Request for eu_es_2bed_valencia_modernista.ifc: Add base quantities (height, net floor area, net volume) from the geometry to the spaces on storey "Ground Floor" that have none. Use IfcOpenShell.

First a look at what the model holds.

```python
import ifcopenshell
import ifcopenshell.util.element
import ifcopenshell.util.unit

model = ifcopenshell.open("eu_es_2bed_valencia_modernista.ifc")
print(model.schema)
for unit_type in ("LENGTHUNIT", "AREAUNIT", "VOLUMEUNIT"):
    print(unit_type, ifcopenshell.util.unit.calculate_unit_scale(model, unit_type))
storey = next(s for s in model.by_type("IfcBuildingStorey") if s.Name == "Ground Floor")
spaces = [e for e in ifcopenshell.util.element.get_decomposition(storey) if e.is_a("IfcSpace")]
for e in sorted(spaces, key=lambda e: e.id()):
    print(e.id(), e.is_a(), e.Name, list(ifcopenshell.util.element.get_psets(e, qtos_only=True)), sep=" | ")
```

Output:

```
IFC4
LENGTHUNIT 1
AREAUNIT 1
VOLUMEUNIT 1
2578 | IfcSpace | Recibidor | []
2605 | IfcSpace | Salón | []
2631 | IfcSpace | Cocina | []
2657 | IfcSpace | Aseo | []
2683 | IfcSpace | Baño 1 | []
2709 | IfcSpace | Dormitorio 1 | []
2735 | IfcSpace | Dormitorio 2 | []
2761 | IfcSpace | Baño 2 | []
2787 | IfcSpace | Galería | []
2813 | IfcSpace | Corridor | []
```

```python
import ifcopenshell
import ifcopenshell.api.pset
import ifcopenshell.geom
import ifcopenshell.util.element
import ifcopenshell.util.shape
import ifcopenshell.util.unit

model = ifcopenshell.open("eu_es_2bed_valencia_modernista.ifc")
unit_scale = ifcopenshell.util.unit.calculate_unit_scale(model)
area_scale = ifcopenshell.util.unit.calculate_unit_scale(model, "AREAUNIT")
volume_scale = ifcopenshell.util.unit.calculate_unit_scale(model, "VOLUMEUNIT")
settings = ifcopenshell.geom.settings()

storey = next(s for s in model.by_type("IfcBuildingStorey") if s.Name == "Ground Floor")
spaces = [e for e in ifcopenshell.util.element.get_decomposition(storey) if e.is_a("IfcSpace")]

for e in sorted(spaces, key=lambda e: e.id()):
    if ifcopenshell.util.element.get_psets(e, qtos_only=True, should_inherit=False):
        continue
    # Geometry comes back in metres, in the element's own axes.
    shape = ifcopenshell.geom.create_shape(settings, e)
    values = {
        "Height": ifcopenshell.util.shape.get_z(shape.geometry) / unit_scale,
        "NetFloorArea": ifcopenshell.util.shape.get_footprint_area(shape.geometry) / area_scale,
        "NetVolume": ifcopenshell.util.shape.get_volume(shape.geometry) / volume_scale,
    }
    qto = ifcopenshell.api.pset.add_qto(model, product=e, name="Qto_SpaceBaseQuantities")
    ifcopenshell.api.pset.edit_qto(model, qto=qto, properties=values)
    print(e.id(), {k: round(v, 3) for k, v in values.items()})

model.write("eu_es_2bed_valencia_modernista_edited.ifc")
```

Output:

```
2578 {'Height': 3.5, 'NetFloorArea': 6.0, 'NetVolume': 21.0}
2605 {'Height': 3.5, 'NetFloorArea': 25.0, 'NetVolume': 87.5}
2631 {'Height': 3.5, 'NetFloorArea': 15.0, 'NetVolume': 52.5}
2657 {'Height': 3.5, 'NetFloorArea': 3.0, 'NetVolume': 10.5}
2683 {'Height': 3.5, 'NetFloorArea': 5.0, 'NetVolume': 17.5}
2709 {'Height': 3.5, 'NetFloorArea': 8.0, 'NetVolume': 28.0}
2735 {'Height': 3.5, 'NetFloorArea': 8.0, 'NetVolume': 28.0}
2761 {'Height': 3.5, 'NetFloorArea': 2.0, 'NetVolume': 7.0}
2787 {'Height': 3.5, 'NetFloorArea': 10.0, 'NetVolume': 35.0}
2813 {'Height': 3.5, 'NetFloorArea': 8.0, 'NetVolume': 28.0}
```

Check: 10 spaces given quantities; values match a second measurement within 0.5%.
